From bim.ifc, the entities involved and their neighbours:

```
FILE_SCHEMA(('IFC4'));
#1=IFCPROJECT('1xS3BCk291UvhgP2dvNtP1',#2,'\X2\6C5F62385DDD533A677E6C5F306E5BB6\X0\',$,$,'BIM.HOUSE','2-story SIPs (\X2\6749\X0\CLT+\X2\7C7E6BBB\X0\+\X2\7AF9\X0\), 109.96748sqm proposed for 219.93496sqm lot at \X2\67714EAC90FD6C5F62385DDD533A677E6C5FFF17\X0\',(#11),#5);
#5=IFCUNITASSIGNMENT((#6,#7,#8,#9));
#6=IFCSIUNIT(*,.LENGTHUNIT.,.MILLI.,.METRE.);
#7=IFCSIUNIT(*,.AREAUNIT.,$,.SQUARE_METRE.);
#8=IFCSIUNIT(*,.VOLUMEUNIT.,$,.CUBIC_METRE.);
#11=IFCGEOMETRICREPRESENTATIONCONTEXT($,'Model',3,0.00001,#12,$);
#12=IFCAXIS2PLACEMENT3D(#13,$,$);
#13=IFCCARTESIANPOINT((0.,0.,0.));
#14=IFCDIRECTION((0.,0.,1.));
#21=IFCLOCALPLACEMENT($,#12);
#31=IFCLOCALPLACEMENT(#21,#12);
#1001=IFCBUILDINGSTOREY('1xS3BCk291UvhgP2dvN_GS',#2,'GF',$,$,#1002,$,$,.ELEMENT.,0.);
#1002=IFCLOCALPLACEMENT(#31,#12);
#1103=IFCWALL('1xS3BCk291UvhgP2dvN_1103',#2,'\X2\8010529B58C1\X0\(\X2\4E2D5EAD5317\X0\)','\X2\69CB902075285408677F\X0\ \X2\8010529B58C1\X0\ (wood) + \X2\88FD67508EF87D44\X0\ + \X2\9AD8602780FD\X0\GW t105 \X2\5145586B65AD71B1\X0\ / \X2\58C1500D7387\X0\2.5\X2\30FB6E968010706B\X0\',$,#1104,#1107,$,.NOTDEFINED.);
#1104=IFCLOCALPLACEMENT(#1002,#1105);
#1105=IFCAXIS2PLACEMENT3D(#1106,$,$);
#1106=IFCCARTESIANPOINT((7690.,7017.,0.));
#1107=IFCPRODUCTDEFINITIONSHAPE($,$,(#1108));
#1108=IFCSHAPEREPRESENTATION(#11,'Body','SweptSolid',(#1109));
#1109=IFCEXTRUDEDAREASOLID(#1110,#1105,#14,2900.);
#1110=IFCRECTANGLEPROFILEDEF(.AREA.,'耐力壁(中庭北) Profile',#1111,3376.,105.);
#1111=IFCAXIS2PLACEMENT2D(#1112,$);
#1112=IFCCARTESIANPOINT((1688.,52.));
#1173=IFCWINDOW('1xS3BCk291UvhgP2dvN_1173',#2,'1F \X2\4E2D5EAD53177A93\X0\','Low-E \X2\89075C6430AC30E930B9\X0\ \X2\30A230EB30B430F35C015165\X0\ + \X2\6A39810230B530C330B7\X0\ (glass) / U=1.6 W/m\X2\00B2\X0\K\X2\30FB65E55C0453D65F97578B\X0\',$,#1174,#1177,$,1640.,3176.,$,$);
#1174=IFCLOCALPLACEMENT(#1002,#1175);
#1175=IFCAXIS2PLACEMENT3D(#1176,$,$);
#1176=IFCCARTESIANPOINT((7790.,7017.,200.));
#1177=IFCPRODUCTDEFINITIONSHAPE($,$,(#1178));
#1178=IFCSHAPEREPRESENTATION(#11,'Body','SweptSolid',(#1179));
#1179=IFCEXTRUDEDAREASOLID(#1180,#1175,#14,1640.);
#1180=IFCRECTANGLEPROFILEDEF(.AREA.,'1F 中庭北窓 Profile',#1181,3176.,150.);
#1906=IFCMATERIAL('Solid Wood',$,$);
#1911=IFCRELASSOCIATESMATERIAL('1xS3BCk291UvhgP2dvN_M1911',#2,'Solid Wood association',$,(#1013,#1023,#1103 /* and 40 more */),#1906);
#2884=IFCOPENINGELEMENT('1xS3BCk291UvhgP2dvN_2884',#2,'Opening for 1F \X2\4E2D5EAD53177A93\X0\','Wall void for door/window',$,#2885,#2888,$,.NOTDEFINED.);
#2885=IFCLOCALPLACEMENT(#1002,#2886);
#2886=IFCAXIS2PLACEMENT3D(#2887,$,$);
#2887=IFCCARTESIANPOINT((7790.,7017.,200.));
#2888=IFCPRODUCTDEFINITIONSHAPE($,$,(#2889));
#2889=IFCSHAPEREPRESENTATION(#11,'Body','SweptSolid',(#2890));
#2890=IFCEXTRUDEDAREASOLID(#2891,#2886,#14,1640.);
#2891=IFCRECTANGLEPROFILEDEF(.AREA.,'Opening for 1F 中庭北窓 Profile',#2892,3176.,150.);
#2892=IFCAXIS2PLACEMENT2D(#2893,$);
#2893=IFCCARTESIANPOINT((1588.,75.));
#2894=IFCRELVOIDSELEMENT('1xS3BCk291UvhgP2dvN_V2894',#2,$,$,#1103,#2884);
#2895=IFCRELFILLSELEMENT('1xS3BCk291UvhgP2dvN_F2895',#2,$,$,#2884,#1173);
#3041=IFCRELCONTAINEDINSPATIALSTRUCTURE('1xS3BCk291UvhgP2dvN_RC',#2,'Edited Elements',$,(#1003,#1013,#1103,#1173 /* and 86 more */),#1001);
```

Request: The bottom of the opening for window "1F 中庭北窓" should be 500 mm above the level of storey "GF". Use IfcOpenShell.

```python
import numpy as np
import ifcopenshell
import ifcopenshell.api.geometry
import ifcopenshell.geom
import ifcopenshell.util.element
import ifcopenshell.util.placement
import ifcopenshell.util.shape
import ifcopenshell.util.unit

model = ifcopenshell.open("bim.ifc")
unit_scale = ifcopenshell.util.unit.calculate_unit_scale(model)

window = model.by_id(1173)
opening = window.FillsVoids[0].RelatingOpeningElement
storey = ifcopenshell.util.element.get_container(window, ifc_class="IfcBuildingStorey")
level = ifcopenshell.util.placement.get_local_placement(storey.ObjectPlacement)[2, 3]

# The opening's origin need not be at the sill, so measure its lowest point.
shape = ifcopenshell.geom.create_shape(ifcopenshell.geom.settings(), opening)
bottom = ifcopenshell.util.shape.get_shape_bottom_elevation(shape, shape.geometry) / unit_scale
dz = level + 0.5 / unit_scale - bottom

shift = np.array([0.0, 0.0, dz])
# The window is not placed relative to its opening, so move both.
for product in (opening, window):
    matrix = ifcopenshell.util.placement.get_local_placement(product.ObjectPlacement)
    matrix[:3, 3] += shift
    ifcopenshell.api.geometry.edit_object_placement(model, product=product, matrix=matrix, is_si=False)

print(f"moved by {dz * unit_scale:+.3f} m")

model.write("bim_rev.ifc")
```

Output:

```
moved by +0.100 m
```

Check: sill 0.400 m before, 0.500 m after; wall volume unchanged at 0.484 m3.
